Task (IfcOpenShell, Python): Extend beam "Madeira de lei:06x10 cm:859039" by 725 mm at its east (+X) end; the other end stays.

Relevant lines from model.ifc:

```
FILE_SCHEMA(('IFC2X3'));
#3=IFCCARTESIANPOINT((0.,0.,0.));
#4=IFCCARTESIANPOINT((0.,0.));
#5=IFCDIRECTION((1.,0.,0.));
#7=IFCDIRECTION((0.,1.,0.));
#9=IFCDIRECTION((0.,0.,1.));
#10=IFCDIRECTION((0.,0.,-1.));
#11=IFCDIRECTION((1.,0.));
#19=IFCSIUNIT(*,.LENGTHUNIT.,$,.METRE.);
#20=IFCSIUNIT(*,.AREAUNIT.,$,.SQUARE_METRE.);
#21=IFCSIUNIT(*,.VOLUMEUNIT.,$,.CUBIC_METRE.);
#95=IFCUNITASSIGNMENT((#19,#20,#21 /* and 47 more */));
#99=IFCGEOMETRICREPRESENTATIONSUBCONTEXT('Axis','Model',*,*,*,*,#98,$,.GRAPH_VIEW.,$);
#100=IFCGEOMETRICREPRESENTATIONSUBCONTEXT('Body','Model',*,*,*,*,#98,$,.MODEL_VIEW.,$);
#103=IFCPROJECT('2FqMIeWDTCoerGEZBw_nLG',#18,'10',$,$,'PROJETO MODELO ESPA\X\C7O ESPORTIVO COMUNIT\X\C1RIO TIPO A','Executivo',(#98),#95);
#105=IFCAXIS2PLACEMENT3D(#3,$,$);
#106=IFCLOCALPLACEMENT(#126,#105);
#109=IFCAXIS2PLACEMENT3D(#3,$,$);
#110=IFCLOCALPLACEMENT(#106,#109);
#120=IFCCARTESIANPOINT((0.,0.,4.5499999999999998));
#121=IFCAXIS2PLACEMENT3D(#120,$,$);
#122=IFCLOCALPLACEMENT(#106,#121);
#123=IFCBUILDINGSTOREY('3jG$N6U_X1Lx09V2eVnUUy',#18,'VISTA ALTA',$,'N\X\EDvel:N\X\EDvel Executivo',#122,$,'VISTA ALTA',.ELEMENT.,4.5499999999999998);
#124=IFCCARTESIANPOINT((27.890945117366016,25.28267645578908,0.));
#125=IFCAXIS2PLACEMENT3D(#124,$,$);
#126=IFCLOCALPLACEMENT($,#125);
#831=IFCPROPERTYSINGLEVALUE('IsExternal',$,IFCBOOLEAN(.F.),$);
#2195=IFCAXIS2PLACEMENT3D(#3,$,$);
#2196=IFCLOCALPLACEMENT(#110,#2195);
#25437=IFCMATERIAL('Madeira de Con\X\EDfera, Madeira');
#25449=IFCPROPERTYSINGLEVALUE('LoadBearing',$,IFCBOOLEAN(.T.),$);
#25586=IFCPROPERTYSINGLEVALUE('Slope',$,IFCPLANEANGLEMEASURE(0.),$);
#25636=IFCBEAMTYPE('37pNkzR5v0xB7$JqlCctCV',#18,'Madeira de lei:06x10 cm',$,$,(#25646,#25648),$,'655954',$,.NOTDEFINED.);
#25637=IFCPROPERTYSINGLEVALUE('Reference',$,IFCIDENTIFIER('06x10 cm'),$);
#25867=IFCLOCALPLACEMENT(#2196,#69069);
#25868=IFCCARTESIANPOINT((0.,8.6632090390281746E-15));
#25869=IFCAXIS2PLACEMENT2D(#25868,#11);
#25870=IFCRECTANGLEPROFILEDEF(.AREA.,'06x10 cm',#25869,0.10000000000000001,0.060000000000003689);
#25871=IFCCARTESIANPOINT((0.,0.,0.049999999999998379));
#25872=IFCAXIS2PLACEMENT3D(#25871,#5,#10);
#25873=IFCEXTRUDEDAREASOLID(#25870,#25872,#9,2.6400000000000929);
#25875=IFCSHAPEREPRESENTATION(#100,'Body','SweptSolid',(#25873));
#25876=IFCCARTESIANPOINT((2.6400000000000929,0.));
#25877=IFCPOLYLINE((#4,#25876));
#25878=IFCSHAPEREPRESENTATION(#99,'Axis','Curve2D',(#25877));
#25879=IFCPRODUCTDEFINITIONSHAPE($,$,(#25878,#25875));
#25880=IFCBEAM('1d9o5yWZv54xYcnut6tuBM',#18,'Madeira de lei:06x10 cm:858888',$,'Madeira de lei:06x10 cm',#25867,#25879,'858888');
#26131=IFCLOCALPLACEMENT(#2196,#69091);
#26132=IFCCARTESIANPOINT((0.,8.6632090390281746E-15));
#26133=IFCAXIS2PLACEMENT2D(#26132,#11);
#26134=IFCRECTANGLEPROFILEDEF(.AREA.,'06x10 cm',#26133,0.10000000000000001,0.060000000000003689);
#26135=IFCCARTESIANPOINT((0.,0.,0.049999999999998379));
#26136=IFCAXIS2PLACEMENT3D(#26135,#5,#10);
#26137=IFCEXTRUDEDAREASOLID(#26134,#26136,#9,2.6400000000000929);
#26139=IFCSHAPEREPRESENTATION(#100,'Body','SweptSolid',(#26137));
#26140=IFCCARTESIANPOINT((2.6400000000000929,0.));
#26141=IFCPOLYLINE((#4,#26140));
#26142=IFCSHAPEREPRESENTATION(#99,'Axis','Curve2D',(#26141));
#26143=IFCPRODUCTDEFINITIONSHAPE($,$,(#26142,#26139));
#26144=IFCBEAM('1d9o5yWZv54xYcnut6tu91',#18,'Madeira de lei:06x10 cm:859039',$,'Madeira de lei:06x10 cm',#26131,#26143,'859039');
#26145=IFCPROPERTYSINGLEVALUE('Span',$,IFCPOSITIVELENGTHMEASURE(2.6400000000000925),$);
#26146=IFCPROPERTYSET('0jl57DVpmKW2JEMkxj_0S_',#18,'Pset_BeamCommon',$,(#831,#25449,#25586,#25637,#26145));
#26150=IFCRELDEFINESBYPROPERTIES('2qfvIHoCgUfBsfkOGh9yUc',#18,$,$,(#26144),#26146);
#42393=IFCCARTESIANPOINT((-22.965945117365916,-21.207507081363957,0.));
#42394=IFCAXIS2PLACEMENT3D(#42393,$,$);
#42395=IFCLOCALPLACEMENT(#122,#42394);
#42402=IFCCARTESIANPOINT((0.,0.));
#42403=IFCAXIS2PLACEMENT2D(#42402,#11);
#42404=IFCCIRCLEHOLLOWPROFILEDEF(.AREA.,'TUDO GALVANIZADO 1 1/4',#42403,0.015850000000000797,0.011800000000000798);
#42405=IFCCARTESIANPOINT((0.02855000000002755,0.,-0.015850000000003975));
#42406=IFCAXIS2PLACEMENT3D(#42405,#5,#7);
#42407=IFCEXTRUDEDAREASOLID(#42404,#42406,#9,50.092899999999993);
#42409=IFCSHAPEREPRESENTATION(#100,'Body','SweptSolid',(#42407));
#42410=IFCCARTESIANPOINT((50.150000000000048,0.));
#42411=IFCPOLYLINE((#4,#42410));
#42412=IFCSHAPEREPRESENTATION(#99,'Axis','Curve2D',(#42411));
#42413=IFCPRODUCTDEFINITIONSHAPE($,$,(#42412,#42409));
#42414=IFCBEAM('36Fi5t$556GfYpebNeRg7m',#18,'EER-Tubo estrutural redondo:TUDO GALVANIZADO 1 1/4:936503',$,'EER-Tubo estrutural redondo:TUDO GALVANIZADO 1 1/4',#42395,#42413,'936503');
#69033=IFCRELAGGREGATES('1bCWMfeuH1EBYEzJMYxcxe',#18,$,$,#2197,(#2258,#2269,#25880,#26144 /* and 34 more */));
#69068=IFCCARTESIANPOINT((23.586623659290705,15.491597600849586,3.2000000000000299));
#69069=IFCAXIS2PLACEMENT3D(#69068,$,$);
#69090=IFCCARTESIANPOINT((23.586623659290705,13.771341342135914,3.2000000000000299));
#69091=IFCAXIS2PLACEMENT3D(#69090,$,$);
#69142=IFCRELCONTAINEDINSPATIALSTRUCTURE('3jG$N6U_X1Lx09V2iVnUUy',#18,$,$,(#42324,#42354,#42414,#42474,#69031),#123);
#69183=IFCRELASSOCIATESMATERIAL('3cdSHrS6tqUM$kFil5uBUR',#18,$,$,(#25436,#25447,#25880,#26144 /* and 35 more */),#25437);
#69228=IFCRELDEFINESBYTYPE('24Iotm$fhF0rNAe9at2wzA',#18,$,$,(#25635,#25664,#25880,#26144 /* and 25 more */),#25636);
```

```python
import numpy as np
import ifcopenshell
import ifcopenshell.api.pset
import ifcopenshell.util.element
import ifcopenshell.util.representation
import ifcopenshell.util.unit

model = ifcopenshell.open("model.ifc")
unit_scale = ifcopenshell.util.unit.calculate_unit_scale(model)

member = model.by_guid("1d9o5yWZv54xYcnut6tu91")
change = 0.725 / unit_scale

# The extrusion runs towards the end named, so only its depth changes.
body = ifcopenshell.util.representation.get_representation(member, "Model", "Body")
solid = body.Items[0]
old_length = solid.Depth
solid.Depth += change

# Move the axis end point with it.
axis = next(r for r in member.Representation.Representations if r.RepresentationIdentifier == "Axis").Items[0]
start, end = (np.array(p.Coordinates) for p in axis.Points)
end = end + (end - start) / np.linalg.norm(end - start) * change
point = model.createIfcCartesianPoint(end.tolist())
axis.Points = [axis.Points[0], point]

# Update the stored length and volume.
pset = model.by_id(ifcopenshell.util.element.get_pset(member, "Pset_BeamCommon", should_inherit=False)["id"])
ifcopenshell.api.pset.edit_pset(model, pset=pset, properties={
    "Span": model.create_entity("IfcPositiveLengthMeasure", solid.Depth),
})

print(f"length {old_length:g} -> {solid.Depth:g}")

model.write("model_rev.ifc")
```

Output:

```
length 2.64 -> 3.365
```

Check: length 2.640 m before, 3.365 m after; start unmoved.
